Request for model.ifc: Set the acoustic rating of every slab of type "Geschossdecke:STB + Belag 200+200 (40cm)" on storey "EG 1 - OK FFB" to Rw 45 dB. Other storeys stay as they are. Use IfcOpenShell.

First a look at what the model holds.

```python
import ifcopenshell
import ifcopenshell.util.element

model = ifcopenshell.open("model.ifc")
print(model.schema)
storey = next(s for s in model.by_type("IfcBuildingStorey") if s.Name == "EG 1 - OK FFB")
slabs = [e for e in ifcopenshell.util.element.get_decomposition(storey) if e.is_a("IfcSlab")]
seen = {}
for e in slabs:
    element_type = ifcopenshell.util.element.get_type(e)
    key = (element_type.Name if element_type != e and element_type else None, ifcopenshell.util.element.get_pset(e, "Pset_SlabCommon", "AcousticRating"))
    seen[key] = seen.get(key, 0) + 1
for (name, value), count in sorted(seen.items(), key=str):
    print(count, "x", name, "|", value)
```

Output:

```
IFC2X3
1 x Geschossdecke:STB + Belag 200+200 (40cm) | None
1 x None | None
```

```python
import ifcopenshell
import ifcopenshell.api.pset
import ifcopenshell.util.element

model = ifcopenshell.open("model.ifc")

storey = next(s for s in model.by_type("IfcBuildingStorey") if s.Name == "EG 1 - OK FFB")
slabs = [e for e in ifcopenshell.util.element.get_decomposition(storey) if e.is_a("IfcSlab")]

count = 0
for e in slabs:
    element_type = ifcopenshell.util.element.get_type(e)
    if element_type in (None, e) or element_type.Name != "Geschossdecke:STB + Belag 200+200 (40cm)":
        continue
    # add_pset returns the element's existing set when there is one.
    pset = ifcopenshell.api.pset.add_pset(model, product=e, name="Pset_SlabCommon")
    ifcopenshell.api.pset.edit_pset(model, pset=pset, properties={"AcousticRating": "Rw 45 dB"})
    count += 1

print(count, "slabs updated")

model.write("model_updated.ifc")
```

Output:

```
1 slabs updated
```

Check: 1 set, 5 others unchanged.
